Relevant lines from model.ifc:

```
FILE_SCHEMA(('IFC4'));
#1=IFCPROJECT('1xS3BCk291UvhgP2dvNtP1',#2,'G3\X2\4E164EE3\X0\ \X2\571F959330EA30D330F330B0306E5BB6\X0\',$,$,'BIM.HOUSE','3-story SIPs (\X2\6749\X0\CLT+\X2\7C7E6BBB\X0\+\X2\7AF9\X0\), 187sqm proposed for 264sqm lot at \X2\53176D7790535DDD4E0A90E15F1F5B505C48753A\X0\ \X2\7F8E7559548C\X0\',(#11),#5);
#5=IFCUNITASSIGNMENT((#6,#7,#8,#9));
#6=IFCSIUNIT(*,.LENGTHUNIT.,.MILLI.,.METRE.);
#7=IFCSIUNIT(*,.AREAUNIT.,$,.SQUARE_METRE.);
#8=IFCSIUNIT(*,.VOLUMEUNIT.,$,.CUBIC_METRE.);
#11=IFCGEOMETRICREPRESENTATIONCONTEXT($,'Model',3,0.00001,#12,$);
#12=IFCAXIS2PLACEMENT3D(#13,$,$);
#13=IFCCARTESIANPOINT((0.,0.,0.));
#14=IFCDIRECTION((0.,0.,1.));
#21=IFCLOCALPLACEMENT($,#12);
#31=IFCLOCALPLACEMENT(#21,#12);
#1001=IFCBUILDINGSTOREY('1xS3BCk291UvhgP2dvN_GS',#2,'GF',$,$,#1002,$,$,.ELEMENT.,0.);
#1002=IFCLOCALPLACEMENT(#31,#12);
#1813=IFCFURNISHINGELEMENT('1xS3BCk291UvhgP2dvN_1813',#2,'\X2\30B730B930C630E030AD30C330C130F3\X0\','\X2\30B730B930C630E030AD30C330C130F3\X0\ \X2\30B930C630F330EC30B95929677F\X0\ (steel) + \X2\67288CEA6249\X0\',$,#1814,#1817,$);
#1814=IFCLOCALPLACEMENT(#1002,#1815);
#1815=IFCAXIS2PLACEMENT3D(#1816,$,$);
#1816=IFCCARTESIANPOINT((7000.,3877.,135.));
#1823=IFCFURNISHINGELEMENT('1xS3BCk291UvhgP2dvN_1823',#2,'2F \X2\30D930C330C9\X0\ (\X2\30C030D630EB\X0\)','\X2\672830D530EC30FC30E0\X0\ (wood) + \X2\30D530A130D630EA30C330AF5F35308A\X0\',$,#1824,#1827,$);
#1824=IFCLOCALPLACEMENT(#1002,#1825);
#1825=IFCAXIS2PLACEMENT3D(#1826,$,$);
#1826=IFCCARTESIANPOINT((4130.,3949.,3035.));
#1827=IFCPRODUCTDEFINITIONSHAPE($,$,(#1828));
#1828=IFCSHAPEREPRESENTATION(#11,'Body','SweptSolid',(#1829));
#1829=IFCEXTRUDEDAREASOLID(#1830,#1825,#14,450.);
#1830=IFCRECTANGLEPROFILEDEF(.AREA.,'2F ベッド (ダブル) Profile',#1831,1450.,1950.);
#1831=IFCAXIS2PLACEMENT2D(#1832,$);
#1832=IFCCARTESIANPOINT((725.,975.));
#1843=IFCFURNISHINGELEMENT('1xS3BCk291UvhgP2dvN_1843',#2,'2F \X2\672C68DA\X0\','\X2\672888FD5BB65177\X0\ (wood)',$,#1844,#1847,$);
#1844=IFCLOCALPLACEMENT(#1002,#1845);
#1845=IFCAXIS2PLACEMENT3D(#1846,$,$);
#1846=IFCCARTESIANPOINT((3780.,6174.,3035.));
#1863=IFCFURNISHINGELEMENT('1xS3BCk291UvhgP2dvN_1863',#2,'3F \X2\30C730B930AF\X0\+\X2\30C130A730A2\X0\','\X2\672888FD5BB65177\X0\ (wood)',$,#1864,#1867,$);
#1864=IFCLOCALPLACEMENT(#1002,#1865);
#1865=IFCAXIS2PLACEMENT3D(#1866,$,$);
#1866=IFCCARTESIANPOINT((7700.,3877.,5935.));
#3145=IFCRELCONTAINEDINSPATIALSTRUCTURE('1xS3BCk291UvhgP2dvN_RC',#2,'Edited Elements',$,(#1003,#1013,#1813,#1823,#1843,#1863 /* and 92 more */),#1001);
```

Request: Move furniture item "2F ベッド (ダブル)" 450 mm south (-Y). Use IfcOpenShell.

```python
import ifcopenshell
import ifcopenshell.api.geometry
import ifcopenshell.util.placement

model = ifcopenshell.open("model.ifc")

item = model.by_id(1823)
matrix = ifcopenshell.util.placement.get_local_placement(item.ObjectPlacement)
matrix[1, 3] -= 450.0
ifcopenshell.api.geometry.edit_object_placement(model, product=item, matrix=matrix, is_si=False)

print(ifcopenshell.util.placement.get_local_placement(item.ObjectPlacement).round(3) + 0.0)

model.write("model_rev.ifc")
```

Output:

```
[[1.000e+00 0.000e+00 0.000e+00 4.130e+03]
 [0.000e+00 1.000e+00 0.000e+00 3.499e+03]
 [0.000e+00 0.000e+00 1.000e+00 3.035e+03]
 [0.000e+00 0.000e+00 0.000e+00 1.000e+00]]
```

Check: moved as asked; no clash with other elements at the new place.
